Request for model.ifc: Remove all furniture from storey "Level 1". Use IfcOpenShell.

First a look at what the model holds.

```python
import ifcopenshell
import ifcopenshell.util.element

model = ifcopenshell.open("model.ifc")
print(model.schema)
storey = next(s for s in model.by_type("IfcBuildingStorey") if s.Name == "Level 1")
furniture = [e for e in ifcopenshell.util.element.get_decomposition(storey) if e.is_a("IfcFurnishingElement")]
seen = {}
for e in furniture:
    element_type = ifcopenshell.util.element.get_type(e)
    name = element_type.Name if element_type not in (None, e) else None
    seen[name] = seen.get(name, 0) + 1
for name, count in sorted(seen.items(), key=str):
    print(count, "x", name)
```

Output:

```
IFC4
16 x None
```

```python
import ifcopenshell
import ifcopenshell.api.root
import ifcopenshell.util.element

model = ifcopenshell.open("model.ifc")

storey = next(s for s in model.by_type("IfcBuildingStorey") if s.Name == "Level 1")
furniture = [e for e in ifcopenshell.util.element.get_decomposition(storey) if e.is_a("IfcFurnishingElement")]

for e in furniture:
    ifcopenshell.api.root.remove_product(model, product=e)
print(len(furniture), "removed")

model.write("model_rev.ifc")
```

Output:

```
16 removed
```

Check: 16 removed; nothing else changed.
